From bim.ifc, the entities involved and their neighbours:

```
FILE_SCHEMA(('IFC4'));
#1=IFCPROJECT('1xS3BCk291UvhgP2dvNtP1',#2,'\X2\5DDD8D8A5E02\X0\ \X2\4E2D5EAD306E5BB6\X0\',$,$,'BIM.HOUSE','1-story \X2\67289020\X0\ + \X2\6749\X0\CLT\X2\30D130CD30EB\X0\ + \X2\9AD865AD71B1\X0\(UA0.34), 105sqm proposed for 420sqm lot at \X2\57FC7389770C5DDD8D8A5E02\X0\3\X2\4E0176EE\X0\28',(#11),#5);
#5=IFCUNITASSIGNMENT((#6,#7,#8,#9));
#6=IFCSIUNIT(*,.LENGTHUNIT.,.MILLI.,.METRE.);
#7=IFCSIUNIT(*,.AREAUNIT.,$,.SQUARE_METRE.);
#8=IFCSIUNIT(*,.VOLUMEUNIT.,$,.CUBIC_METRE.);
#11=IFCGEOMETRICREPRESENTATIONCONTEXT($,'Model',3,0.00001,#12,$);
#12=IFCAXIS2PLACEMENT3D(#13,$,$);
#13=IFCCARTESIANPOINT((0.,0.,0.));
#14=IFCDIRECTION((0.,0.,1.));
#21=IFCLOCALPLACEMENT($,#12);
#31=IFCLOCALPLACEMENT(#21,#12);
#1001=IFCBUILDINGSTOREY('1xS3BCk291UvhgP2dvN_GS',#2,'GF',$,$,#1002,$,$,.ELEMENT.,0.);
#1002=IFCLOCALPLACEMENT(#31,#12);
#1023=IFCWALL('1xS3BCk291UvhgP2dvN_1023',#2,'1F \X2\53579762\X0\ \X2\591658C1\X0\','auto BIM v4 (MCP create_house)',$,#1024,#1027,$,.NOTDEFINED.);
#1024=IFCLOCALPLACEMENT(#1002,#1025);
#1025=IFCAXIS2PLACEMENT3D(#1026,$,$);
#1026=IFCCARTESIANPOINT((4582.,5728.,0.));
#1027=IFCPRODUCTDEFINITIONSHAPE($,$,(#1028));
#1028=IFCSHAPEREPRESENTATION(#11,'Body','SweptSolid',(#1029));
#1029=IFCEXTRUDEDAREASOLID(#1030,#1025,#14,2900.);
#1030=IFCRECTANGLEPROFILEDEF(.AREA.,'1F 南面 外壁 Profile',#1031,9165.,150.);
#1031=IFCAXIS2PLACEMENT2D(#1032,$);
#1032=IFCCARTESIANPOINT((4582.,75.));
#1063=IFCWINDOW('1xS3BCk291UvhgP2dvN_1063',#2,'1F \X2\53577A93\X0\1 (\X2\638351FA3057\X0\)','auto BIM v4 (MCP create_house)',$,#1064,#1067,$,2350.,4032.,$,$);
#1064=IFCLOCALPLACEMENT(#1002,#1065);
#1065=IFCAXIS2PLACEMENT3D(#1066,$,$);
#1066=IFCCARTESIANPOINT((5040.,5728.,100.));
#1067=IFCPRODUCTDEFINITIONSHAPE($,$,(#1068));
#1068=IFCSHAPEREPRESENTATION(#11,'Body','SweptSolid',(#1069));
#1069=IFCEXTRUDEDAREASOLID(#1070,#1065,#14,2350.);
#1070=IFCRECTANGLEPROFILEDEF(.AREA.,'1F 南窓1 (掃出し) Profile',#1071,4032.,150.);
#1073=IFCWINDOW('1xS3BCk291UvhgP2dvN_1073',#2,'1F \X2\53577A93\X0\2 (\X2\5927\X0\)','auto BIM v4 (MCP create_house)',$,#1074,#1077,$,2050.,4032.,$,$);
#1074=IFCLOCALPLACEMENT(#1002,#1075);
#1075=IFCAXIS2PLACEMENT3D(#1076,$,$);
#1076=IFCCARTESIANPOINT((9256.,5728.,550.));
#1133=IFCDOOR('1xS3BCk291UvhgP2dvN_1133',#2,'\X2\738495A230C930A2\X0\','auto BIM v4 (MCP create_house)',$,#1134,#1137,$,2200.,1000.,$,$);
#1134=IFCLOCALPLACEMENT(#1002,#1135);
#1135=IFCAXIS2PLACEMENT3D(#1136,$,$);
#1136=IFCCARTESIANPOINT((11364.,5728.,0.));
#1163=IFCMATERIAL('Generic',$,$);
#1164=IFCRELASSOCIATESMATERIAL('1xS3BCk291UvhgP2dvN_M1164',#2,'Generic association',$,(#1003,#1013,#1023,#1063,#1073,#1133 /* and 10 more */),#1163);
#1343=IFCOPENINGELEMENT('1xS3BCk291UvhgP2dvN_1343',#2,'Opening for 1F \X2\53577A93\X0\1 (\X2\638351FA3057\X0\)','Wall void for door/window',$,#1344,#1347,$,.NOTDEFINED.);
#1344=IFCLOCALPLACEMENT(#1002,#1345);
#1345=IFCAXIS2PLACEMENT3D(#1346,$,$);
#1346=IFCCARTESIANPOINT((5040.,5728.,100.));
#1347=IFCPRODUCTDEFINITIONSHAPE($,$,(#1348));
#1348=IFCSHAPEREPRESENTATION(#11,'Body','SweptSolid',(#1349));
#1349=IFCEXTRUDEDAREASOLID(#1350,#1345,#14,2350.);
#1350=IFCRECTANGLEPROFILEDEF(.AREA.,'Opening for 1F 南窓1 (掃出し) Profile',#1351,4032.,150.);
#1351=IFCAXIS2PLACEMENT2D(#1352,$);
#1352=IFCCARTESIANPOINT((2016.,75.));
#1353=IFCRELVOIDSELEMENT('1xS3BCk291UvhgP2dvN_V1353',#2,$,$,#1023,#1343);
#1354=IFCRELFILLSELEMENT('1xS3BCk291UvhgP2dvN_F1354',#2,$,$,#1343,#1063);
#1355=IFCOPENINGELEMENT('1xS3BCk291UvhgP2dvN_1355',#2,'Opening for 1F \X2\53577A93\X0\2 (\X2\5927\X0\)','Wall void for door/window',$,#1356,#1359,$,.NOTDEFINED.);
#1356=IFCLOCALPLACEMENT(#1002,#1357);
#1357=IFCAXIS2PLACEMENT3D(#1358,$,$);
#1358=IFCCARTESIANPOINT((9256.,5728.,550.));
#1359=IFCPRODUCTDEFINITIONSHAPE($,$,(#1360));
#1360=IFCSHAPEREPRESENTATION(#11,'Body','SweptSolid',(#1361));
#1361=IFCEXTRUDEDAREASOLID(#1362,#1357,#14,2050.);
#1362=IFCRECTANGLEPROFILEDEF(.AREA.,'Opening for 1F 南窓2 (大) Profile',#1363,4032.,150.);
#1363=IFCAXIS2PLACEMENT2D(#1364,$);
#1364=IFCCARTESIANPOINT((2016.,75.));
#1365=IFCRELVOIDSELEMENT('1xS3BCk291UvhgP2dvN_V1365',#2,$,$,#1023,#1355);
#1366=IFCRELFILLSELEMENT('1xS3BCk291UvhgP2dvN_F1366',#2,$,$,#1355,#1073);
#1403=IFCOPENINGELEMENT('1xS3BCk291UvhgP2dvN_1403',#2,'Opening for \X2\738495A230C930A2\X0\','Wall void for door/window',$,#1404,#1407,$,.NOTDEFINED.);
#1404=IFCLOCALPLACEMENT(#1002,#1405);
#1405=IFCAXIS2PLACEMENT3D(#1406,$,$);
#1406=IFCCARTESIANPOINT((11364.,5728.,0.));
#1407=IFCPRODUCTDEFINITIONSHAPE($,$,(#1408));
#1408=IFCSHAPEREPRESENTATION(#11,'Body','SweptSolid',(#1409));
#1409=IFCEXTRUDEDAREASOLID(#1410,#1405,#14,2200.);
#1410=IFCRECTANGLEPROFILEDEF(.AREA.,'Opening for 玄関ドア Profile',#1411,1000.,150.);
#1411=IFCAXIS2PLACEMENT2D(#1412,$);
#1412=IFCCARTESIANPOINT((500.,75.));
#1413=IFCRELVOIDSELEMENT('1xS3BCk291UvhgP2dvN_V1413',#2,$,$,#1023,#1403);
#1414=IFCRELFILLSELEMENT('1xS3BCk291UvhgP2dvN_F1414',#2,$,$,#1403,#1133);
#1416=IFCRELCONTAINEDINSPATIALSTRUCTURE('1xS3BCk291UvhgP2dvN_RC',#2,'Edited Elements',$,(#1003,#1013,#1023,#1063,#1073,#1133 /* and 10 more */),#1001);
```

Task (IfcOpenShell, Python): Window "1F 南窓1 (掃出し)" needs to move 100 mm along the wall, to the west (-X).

```python
import ifcopenshell
import ifcopenshell.api.geometry
import ifcopenshell.util.placement

model = ifcopenshell.open("bim.ifc")

window = model.by_id(1063)
opening = window.FillsVoids[0].RelatingOpeningElement
wall = opening.VoidsElements[0].RelatingBuildingElement

wall_matrix = ifcopenshell.util.placement.get_local_placement(wall.ObjectPlacement)
shift = wall_matrix[:3, 0] * -100.0
before = ifcopenshell.util.placement.get_local_placement(window.ObjectPlacement)[:3, 3].copy()

# The window is not placed relative to its opening, so move both.
for product in (opening, window):
    matrix = ifcopenshell.util.placement.get_local_placement(product.ObjectPlacement)
    matrix[:3, 3] += shift
    ifcopenshell.api.geometry.edit_object_placement(model, product=product, matrix=matrix, is_si=False)

after = ifcopenshell.util.placement.get_local_placement(window.ObjectPlacement)[:3, 3]
print("window moved by", (after - before).round(3) + 0.0)

model.write("bim-out.ifc")
```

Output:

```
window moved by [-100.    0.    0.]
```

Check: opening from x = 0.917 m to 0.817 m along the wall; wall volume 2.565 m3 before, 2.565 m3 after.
